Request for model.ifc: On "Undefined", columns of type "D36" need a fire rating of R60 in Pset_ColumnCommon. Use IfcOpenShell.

First a look at what the model holds.

```python
import ifcopenshell
import ifcopenshell.util.element

model = ifcopenshell.open("model.ifc")
print(model.schema)
storey = next(s for s in model.by_type("IfcBuildingStorey") if s.Name == "Undefined")
columns = [e for e in ifcopenshell.util.element.get_decomposition(storey) if e.is_a("IfcColumn")]
seen = {}
for e in columns:
    element_type = ifcopenshell.util.element.get_type(e)
    key = (element_type.Name if element_type != e and element_type else None, ifcopenshell.util.element.get_pset(e, "Pset_ColumnCommon", "FireRating"))
    seen[key] = seen.get(key, 0) + 1
for (name, value), count in sorted(seen.items(), key=str):
    print(count, "x", name, "|", value)
```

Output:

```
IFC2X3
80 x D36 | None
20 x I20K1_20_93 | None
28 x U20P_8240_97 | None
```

```python
import ifcopenshell
import ifcopenshell.api.pset
import ifcopenshell.util.element

model = ifcopenshell.open("model.ifc")

storey = next(s for s in model.by_type("IfcBuildingStorey") if s.Name == "Undefined")
columns = [e for e in ifcopenshell.util.element.get_decomposition(storey) if e.is_a("IfcColumn")]

count = 0
for e in columns:
    element_type = ifcopenshell.util.element.get_type(e)
    if element_type in (None, e) or element_type.Name != "D36":
        continue
    found = ifcopenshell.util.element.get_pset(e, "Pset_ColumnCommon", should_inherit=False)
    if found:
        pset = model.by_id(found["id"])
        if len(ifcopenshell.util.element.get_elements_by_pset(pset)) > 1:
            pset = ifcopenshell.api.pset.unshare_pset(model, products=[e], pset=pset)[0]
    else:
        pset = ifcopenshell.api.pset.add_pset(model, product=e, name="Pset_ColumnCommon")
    ifcopenshell.api.pset.edit_pset(model, pset=pset, properties={"FireRating": "R60"})
    count += 1

print(count, "columns updated")

model.write("model_updated.ifc")
```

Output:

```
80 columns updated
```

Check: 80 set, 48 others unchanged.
